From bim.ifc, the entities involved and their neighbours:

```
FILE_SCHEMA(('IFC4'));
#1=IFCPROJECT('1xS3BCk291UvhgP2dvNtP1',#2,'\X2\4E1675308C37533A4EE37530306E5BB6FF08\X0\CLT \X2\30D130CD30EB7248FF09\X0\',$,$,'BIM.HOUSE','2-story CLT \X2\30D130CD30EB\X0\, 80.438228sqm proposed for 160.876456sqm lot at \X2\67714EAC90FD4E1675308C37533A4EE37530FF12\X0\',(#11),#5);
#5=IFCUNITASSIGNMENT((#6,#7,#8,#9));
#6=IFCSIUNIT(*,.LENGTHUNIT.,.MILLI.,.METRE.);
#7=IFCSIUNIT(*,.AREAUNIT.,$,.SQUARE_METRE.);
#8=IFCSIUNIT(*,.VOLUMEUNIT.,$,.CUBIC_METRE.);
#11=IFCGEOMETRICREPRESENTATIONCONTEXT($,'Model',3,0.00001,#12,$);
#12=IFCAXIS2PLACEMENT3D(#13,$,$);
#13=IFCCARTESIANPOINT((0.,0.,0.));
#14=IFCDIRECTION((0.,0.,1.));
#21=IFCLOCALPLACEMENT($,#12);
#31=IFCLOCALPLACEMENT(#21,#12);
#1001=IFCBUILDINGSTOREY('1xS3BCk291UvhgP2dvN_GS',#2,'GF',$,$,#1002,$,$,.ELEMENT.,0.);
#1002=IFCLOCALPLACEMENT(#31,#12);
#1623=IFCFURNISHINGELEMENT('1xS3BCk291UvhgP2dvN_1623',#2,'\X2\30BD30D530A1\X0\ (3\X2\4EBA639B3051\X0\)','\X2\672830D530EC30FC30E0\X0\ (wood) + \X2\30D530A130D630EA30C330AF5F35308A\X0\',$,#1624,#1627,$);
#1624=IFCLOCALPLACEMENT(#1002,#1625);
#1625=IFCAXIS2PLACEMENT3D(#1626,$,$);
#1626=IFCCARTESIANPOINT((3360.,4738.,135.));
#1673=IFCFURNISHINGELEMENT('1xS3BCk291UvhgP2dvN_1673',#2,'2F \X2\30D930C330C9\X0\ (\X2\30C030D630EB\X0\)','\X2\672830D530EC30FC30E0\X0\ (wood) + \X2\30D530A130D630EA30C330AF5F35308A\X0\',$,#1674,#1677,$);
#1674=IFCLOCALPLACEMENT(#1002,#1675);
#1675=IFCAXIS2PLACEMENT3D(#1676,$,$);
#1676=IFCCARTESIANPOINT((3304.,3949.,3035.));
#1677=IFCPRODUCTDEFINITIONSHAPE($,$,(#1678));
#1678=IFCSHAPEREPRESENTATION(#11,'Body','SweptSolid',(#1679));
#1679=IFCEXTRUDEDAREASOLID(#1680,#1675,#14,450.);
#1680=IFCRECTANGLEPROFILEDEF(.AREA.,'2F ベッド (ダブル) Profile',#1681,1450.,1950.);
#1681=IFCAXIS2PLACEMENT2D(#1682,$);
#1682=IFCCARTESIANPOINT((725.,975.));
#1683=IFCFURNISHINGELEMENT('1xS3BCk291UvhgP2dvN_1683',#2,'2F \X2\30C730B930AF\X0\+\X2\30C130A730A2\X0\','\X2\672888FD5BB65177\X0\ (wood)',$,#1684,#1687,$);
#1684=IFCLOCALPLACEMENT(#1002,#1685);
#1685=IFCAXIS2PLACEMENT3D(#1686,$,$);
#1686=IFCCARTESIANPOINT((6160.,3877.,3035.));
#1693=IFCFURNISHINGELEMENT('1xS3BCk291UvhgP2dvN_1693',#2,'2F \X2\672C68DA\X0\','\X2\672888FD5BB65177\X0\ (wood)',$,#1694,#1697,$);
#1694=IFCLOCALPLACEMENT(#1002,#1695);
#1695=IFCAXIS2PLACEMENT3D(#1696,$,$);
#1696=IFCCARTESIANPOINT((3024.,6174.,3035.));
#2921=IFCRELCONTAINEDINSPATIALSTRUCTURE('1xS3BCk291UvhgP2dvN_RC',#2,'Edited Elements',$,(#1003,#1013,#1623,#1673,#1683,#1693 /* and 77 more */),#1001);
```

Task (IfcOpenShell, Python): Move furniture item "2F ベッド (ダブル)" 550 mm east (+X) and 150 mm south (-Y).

```python
import ifcopenshell
import ifcopenshell.api.geometry
import ifcopenshell.util.placement
import ifcopenshell.util.unit

model = ifcopenshell.open("bim.ifc")
unit_scale = ifcopenshell.util.unit.calculate_unit_scale(model)

item = model.by_guid("1xS3BCk291UvhgP2dvN_1673")
matrix = ifcopenshell.util.placement.get_local_placement(item.ObjectPlacement)
matrix[0, 3] += 0.55 / unit_scale
matrix[1, 3] -= 0.15 / unit_scale
ifcopenshell.api.geometry.edit_object_placement(model, product=item, matrix=matrix, is_si=False)

print(ifcopenshell.util.placement.get_local_placement(item.ObjectPlacement).round(3) + 0.0)

model.write("bim_updated.ifc")
```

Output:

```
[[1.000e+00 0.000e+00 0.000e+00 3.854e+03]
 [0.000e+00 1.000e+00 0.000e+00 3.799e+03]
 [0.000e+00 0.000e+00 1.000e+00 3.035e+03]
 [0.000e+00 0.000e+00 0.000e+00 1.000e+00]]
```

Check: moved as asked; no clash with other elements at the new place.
